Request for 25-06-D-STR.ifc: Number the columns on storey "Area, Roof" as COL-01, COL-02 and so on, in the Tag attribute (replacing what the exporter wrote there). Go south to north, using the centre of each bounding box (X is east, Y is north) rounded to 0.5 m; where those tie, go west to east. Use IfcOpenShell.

First a look at what the model holds.

```python
import ifcopenshell
import ifcopenshell.util.element
import ifcopenshell.util.placement

model = ifcopenshell.open("25-06-D-STR.ifc")
print(model.schema)
storey = next(s for s in model.by_type("IfcBuildingStorey") if s.Name == "Area, Roof")
columns = [e for e in ifcopenshell.util.element.get_decomposition(storey) if e.is_a("IfcColumn")]
for e in sorted(columns, key=lambda e: e.id()):
    origin = ifcopenshell.util.placement.get_local_placement(e.ObjectPlacement)[:3, 3]
    print(e.id(), e.Tag, e.Name, origin.round(2) + 0.0, sep=" | ")
```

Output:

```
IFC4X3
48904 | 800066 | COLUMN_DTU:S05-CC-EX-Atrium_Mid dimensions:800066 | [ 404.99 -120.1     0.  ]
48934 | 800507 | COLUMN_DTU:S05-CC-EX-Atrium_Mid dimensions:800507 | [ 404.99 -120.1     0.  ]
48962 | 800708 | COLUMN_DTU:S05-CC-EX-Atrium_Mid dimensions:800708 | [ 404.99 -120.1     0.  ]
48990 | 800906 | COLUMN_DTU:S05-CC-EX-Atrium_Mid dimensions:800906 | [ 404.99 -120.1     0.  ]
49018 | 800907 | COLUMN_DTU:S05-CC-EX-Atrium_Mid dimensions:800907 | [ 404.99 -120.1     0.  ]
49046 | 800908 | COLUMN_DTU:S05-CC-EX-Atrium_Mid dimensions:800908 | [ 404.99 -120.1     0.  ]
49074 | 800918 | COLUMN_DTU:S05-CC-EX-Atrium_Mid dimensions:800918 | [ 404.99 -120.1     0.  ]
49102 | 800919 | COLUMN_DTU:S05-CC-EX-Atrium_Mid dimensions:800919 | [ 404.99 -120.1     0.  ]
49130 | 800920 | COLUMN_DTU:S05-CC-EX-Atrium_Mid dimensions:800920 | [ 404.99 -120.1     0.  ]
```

```python
import ifcopenshell
import ifcopenshell.geom
import ifcopenshell.util.element
import ifcopenshell.util.shape

model = ifcopenshell.open("25-06-D-STR.ifc")
settings = ifcopenshell.geom.settings()
settings.set("use-world-coords", True)


def centre(element):
    shape = ifcopenshell.geom.create_shape(settings, element)
    return ifcopenshell.util.shape.get_bbox_centroid(shape.geometry)


storey = next(s for s in model.by_type("IfcBuildingStorey") if s.Name == "Area, Roof")
columns = [e for e in ifcopenshell.util.element.get_decomposition(storey) if e.is_a("IfcColumn")]

# Insertion points can sit at a corner or the storey origin, so sort by the geometry (in metres).
centres = {e: centre(e) for e in columns}
columns.sort(key=lambda e: (round(centres[e][1] / 0.5), centres[e][0]))

for i, e in enumerate(columns, start=1):
    number = f"COL-{i:02d}"
    e.Tag = number
    print(e.id(), number)

model.write("25-06-D-STR-out.ifc")
```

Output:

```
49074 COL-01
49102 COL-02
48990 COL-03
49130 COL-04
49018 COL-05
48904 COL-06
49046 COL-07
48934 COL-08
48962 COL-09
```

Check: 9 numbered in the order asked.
